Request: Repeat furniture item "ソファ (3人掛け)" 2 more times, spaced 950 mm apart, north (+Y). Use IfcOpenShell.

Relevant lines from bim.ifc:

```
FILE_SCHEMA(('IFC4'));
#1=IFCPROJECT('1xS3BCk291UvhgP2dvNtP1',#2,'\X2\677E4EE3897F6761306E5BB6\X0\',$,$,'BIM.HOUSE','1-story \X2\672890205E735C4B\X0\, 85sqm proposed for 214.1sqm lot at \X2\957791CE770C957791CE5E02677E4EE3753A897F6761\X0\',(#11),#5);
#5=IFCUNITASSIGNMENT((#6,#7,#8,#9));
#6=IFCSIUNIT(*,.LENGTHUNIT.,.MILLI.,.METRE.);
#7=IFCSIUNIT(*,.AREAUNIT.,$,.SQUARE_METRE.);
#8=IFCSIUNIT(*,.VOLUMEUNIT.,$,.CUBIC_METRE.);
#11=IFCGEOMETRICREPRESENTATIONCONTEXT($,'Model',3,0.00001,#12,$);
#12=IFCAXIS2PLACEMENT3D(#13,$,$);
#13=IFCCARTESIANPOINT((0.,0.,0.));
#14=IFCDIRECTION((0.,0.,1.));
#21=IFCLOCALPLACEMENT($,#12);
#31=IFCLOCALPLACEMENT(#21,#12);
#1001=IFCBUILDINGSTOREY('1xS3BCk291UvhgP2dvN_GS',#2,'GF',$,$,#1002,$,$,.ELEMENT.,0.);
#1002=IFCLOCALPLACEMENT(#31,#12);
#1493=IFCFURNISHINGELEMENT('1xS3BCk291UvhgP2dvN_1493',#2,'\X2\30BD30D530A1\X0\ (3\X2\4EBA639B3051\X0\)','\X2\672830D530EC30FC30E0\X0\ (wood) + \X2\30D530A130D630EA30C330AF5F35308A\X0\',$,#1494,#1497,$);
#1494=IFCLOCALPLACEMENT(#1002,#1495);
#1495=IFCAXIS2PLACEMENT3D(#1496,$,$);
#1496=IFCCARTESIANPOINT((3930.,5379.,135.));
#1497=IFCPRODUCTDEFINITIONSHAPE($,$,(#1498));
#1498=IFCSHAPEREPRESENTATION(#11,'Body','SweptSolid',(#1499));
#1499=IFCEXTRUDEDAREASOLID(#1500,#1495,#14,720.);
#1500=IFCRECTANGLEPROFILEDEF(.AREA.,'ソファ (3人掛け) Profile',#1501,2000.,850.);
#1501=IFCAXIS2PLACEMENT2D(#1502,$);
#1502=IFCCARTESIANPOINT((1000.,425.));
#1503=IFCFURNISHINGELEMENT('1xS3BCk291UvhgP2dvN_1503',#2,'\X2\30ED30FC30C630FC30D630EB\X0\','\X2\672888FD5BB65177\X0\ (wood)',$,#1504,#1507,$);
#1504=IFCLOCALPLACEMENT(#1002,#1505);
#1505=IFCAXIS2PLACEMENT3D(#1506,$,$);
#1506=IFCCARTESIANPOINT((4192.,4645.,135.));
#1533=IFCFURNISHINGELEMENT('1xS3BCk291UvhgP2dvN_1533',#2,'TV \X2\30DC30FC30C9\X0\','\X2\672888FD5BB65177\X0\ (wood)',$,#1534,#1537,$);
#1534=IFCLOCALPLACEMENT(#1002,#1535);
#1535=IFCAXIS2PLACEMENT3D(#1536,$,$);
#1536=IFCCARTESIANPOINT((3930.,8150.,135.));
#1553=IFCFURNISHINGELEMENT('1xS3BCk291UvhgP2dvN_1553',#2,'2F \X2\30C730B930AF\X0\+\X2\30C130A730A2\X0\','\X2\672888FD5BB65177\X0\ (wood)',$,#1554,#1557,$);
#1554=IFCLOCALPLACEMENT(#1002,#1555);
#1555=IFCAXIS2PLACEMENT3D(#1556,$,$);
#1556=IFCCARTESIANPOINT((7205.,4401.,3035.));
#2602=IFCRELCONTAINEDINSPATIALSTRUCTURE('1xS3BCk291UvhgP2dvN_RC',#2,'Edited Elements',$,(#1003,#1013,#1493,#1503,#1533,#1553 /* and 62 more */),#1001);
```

```python
import numpy as np
import ifcopenshell
import ifcopenshell.api.geometry
import ifcopenshell.api.root
import ifcopenshell.util.element
import ifcopenshell.util.placement

model = ifcopenshell.open("bim.ifc")


def reuse_history(source, copy):
    """copy_class also copies each property set's owner history, people and application; keep the originals."""
    for rel in copy.IsDefinedBy:
        if rel.is_a("IfcRelDefinesByProperties") and (history := rel.RelatingPropertyDefinition.OwnerHistory):
            rel.RelatingPropertyDefinition.OwnerHistory = source.OwnerHistory
            ifcopenshell.util.element.remove_deep2(model, history)


source = model.by_id(1493)
base = ifcopenshell.util.placement.get_local_placement(source.ObjectPlacement)
step = np.array([0.0, 1.0, 0.0]) * 950.0

for i in range(1, 3):
    copy = ifcopenshell.api.root.copy_class(model, product=source)
    copy.Representation = ifcopenshell.util.element.copy_deep(
        model, source.Representation, exclude=["IfcGeometricRepresentationContext", "IfcRepresentationMap"]
    )
    reuse_history(source, copy)
    matrix = base.copy()
    matrix[:3, 3] += i * step
    print("added at", matrix[:3, 3].round(3) + 0.0)
    ifcopenshell.api.geometry.edit_object_placement(model, product=copy, matrix=matrix, is_si=False)

model.write("bim-out.ifc")
```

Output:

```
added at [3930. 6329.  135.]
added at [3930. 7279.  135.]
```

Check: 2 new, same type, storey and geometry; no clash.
